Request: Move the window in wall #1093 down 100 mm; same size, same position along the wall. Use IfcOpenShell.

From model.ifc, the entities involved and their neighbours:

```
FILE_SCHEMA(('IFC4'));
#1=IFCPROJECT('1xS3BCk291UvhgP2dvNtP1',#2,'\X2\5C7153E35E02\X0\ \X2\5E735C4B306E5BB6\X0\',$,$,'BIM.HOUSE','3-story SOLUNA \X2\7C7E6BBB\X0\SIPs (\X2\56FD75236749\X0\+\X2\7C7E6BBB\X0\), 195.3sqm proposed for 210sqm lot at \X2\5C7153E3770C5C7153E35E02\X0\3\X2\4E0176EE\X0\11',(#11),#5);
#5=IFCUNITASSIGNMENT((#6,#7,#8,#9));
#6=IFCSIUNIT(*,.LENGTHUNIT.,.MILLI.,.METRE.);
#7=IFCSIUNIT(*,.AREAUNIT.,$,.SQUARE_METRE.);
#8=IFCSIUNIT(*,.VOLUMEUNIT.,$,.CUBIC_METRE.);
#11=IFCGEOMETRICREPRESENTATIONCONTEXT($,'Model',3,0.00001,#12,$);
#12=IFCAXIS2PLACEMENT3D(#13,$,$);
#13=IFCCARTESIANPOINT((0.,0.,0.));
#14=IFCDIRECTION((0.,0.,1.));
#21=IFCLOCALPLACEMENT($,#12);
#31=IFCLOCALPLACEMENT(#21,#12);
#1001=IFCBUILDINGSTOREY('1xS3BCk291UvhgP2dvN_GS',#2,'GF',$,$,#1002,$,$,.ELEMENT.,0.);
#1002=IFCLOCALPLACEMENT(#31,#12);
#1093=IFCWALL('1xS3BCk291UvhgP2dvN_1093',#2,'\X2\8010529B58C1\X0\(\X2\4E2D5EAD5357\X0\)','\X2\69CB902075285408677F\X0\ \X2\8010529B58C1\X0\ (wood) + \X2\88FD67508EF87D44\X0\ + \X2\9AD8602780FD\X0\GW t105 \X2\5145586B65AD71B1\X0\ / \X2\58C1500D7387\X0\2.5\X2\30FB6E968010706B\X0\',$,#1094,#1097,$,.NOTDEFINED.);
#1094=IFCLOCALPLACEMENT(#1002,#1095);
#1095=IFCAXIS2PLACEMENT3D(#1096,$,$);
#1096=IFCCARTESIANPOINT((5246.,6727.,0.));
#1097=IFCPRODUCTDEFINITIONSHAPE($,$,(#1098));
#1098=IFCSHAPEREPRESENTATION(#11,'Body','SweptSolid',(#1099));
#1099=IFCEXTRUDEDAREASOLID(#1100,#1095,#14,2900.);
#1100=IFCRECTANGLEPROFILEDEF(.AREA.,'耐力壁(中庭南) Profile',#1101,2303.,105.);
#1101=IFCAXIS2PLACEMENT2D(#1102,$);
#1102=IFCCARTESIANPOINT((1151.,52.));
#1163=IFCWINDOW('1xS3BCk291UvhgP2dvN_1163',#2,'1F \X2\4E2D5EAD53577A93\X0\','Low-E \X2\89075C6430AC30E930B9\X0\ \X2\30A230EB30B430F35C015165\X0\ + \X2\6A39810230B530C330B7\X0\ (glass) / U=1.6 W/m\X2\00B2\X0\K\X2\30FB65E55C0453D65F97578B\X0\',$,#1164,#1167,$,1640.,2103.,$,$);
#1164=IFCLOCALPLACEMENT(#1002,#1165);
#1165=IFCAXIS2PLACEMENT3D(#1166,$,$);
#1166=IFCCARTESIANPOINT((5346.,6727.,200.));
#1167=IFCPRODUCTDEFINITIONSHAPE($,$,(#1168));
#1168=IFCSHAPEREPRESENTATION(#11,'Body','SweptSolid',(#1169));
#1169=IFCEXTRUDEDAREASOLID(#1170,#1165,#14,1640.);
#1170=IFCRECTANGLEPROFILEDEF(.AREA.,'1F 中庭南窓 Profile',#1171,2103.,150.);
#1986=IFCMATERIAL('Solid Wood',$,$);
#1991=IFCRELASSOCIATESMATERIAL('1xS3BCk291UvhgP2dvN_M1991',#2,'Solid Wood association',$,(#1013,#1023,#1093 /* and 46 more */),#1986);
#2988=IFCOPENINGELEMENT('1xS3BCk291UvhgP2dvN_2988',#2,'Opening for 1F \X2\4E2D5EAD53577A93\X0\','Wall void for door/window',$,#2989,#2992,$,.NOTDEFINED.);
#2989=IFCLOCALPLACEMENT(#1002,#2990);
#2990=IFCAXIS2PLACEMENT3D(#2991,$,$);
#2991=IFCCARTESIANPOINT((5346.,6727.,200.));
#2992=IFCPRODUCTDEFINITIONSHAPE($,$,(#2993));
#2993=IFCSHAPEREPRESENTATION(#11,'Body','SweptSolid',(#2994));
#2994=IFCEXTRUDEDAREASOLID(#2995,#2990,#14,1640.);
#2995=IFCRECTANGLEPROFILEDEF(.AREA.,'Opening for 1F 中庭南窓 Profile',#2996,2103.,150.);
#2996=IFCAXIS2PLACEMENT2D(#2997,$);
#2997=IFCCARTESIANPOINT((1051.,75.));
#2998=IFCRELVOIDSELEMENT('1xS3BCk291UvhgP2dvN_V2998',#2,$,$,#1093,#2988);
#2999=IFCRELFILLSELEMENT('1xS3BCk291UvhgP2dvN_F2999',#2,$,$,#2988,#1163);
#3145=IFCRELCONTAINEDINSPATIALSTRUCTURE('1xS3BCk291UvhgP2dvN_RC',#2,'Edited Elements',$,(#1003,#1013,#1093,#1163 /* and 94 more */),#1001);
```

```python
import numpy as np
import ifcopenshell
import ifcopenshell.api.geometry
import ifcopenshell.util.placement
import ifcopenshell.util.unit

model = ifcopenshell.open("model.ifc")
unit_scale = ifcopenshell.util.unit.calculate_unit_scale(model)

window = model.by_guid("1xS3BCk291UvhgP2dvN_1163")
opening = window.FillsVoids[0].RelatingOpeningElement
dz = -100.0

shift = np.array([0.0, 0.0, dz])
# The window is not placed relative to its opening, so move both.
for product in (opening, window):
    matrix = ifcopenshell.util.placement.get_local_placement(product.ObjectPlacement)
    matrix[:3, 3] += shift
    ifcopenshell.api.geometry.edit_object_placement(model, product=product, matrix=matrix, is_si=False)

print(f"moved by {dz * unit_scale:+.3f} m")

model.write("model_updated.ifc")
```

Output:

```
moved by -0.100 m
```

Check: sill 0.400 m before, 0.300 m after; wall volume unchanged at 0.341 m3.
